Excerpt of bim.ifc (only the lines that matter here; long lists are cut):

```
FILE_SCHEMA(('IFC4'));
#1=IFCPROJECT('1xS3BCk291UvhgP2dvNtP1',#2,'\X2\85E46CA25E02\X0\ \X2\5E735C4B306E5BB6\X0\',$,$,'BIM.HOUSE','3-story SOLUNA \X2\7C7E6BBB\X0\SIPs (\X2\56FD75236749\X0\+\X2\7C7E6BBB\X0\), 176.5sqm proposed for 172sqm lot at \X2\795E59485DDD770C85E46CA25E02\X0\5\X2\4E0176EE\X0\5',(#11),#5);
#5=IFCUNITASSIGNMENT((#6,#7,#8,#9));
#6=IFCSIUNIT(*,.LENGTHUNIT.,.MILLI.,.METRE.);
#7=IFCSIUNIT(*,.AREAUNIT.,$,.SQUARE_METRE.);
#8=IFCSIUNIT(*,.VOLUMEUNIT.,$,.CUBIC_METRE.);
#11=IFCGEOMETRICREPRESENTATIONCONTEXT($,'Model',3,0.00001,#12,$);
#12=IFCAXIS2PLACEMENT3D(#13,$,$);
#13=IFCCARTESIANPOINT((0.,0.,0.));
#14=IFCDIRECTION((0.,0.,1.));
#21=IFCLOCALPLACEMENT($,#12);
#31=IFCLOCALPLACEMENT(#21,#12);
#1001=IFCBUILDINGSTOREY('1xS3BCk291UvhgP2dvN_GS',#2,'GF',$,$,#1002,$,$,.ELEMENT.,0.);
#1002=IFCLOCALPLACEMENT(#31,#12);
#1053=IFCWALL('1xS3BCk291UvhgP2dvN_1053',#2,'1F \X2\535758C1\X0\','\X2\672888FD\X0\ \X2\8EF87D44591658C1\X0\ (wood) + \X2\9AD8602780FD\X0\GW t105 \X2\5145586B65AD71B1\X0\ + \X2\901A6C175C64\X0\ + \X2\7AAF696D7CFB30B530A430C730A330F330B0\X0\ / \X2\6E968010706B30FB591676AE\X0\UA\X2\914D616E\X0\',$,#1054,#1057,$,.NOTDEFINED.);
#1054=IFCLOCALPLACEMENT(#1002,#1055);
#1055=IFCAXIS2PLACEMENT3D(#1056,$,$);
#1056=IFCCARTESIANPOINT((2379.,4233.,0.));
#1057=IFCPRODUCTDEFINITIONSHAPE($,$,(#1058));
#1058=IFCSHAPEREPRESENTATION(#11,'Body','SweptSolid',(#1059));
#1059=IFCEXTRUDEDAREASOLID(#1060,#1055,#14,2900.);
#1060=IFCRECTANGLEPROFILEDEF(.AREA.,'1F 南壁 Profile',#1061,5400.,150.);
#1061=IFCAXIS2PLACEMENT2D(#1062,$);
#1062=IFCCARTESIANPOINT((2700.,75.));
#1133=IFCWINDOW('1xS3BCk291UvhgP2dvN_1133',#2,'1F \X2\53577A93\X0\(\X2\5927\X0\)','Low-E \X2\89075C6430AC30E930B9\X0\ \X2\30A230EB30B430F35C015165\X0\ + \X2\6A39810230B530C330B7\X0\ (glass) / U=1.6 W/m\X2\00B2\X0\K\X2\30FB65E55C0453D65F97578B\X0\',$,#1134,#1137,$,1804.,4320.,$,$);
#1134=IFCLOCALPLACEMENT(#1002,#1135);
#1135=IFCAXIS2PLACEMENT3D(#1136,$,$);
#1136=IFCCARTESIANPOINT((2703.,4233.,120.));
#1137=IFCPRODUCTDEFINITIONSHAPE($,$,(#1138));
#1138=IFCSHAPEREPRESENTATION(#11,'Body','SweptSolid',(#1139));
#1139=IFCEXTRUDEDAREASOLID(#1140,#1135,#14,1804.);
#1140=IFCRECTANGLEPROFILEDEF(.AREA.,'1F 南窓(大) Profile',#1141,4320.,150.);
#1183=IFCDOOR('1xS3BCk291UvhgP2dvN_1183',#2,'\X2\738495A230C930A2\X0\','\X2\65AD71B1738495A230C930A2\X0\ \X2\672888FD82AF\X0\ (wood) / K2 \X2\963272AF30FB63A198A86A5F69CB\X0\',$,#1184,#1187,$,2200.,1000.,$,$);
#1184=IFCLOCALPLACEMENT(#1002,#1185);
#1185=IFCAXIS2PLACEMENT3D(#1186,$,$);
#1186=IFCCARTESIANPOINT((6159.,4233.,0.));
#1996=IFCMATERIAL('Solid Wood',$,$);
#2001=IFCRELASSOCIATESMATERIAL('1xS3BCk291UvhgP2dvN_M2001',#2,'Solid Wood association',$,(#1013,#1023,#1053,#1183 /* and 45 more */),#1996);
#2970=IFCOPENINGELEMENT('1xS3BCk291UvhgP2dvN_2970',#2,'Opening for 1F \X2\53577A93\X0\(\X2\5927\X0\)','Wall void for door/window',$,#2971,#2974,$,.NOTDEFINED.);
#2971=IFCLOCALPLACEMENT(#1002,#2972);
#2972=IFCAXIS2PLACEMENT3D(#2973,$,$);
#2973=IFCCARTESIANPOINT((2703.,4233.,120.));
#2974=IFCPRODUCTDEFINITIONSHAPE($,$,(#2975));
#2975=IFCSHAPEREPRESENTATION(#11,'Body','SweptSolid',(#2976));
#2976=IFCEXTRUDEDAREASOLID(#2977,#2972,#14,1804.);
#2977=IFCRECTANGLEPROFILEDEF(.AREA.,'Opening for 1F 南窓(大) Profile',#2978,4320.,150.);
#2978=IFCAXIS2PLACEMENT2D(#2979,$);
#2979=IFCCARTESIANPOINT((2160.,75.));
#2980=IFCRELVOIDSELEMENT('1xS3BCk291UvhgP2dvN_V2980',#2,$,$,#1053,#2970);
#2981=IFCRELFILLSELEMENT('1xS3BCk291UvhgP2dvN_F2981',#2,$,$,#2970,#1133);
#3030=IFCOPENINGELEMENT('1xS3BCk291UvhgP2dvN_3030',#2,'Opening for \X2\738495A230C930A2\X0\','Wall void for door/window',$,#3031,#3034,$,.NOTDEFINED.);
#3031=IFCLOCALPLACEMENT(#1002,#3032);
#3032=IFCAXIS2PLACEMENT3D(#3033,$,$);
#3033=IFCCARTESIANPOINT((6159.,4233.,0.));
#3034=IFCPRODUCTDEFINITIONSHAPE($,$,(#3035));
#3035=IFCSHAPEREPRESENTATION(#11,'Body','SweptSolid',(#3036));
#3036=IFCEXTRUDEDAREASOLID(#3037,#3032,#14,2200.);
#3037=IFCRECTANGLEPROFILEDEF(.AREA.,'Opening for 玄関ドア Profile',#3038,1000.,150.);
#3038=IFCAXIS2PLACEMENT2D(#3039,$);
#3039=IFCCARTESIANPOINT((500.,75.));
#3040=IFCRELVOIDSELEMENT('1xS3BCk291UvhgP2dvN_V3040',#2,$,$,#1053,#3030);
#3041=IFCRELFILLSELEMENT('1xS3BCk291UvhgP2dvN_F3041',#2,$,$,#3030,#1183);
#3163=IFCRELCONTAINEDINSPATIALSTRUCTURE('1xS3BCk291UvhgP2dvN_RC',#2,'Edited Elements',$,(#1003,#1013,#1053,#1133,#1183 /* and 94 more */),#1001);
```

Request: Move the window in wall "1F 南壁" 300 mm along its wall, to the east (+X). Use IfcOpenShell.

```python
import ifcopenshell
import ifcopenshell.api.geometry
import ifcopenshell.util.placement

model = ifcopenshell.open("bim.ifc")

window = model.by_id(1133)
opening = window.FillsVoids[0].RelatingOpeningElement
wall = opening.VoidsElements[0].RelatingBuildingElement

wall_matrix = ifcopenshell.util.placement.get_local_placement(wall.ObjectPlacement)
shift = wall_matrix[:3, 0] * 300.0
before = ifcopenshell.util.placement.get_local_placement(window.ObjectPlacement)[:3, 3].copy()

# The window is not placed relative to its opening, so move both.
for product in (opening, window):
    matrix = ifcopenshell.util.placement.get_local_placement(product.ObjectPlacement)
    matrix[:3, 3] += shift
    ifcopenshell.api.geometry.edit_object_placement(model, product=product, matrix=matrix, is_si=False)

after = ifcopenshell.util.placement.get_local_placement(window.ObjectPlacement)[:3, 3]
print("window moved by", (after - before).round(3) + 0.0)

model.write("bim_v2.ifc")
```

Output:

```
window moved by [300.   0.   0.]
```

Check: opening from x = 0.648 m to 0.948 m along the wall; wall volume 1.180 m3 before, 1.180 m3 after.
